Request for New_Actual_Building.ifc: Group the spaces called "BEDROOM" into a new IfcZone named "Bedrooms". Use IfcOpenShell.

First a look at what the model holds.

```python
import ifcopenshell

model = ifcopenshell.open("New_Actual_Building.ifc")
print(model.schema)
seen = {}
for space in model.by_type("IfcSpace"):
    seen[space.LongName] = seen.get(space.LongName, 0) + 1
for name, count in sorted(seen.items(), key=str):
    print(count, "x", name)
print("zones:", [z.Name for z in model.by_type("IfcZone")][:20])
```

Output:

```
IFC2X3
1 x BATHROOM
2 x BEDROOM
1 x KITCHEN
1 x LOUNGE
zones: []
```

```python
import ifcopenshell
import ifcopenshell.api.group
import ifcopenshell.api.root

model = ifcopenshell.open("New_Actual_Building.ifc")

names = {"BEDROOM"}
spaces = [s for s in model.by_type("IfcSpace") if s.LongName in names]

zone = ifcopenshell.api.root.create_entity(model, ifc_class="IfcZone", name="Bedrooms")
ifcopenshell.api.group.assign_group(model, products=spaces, group=zone)
print(len(spaces), "spaces in", zone.Name)

model.write("New_Actual_Building_v2.ifc")
```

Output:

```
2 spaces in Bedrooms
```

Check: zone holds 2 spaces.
